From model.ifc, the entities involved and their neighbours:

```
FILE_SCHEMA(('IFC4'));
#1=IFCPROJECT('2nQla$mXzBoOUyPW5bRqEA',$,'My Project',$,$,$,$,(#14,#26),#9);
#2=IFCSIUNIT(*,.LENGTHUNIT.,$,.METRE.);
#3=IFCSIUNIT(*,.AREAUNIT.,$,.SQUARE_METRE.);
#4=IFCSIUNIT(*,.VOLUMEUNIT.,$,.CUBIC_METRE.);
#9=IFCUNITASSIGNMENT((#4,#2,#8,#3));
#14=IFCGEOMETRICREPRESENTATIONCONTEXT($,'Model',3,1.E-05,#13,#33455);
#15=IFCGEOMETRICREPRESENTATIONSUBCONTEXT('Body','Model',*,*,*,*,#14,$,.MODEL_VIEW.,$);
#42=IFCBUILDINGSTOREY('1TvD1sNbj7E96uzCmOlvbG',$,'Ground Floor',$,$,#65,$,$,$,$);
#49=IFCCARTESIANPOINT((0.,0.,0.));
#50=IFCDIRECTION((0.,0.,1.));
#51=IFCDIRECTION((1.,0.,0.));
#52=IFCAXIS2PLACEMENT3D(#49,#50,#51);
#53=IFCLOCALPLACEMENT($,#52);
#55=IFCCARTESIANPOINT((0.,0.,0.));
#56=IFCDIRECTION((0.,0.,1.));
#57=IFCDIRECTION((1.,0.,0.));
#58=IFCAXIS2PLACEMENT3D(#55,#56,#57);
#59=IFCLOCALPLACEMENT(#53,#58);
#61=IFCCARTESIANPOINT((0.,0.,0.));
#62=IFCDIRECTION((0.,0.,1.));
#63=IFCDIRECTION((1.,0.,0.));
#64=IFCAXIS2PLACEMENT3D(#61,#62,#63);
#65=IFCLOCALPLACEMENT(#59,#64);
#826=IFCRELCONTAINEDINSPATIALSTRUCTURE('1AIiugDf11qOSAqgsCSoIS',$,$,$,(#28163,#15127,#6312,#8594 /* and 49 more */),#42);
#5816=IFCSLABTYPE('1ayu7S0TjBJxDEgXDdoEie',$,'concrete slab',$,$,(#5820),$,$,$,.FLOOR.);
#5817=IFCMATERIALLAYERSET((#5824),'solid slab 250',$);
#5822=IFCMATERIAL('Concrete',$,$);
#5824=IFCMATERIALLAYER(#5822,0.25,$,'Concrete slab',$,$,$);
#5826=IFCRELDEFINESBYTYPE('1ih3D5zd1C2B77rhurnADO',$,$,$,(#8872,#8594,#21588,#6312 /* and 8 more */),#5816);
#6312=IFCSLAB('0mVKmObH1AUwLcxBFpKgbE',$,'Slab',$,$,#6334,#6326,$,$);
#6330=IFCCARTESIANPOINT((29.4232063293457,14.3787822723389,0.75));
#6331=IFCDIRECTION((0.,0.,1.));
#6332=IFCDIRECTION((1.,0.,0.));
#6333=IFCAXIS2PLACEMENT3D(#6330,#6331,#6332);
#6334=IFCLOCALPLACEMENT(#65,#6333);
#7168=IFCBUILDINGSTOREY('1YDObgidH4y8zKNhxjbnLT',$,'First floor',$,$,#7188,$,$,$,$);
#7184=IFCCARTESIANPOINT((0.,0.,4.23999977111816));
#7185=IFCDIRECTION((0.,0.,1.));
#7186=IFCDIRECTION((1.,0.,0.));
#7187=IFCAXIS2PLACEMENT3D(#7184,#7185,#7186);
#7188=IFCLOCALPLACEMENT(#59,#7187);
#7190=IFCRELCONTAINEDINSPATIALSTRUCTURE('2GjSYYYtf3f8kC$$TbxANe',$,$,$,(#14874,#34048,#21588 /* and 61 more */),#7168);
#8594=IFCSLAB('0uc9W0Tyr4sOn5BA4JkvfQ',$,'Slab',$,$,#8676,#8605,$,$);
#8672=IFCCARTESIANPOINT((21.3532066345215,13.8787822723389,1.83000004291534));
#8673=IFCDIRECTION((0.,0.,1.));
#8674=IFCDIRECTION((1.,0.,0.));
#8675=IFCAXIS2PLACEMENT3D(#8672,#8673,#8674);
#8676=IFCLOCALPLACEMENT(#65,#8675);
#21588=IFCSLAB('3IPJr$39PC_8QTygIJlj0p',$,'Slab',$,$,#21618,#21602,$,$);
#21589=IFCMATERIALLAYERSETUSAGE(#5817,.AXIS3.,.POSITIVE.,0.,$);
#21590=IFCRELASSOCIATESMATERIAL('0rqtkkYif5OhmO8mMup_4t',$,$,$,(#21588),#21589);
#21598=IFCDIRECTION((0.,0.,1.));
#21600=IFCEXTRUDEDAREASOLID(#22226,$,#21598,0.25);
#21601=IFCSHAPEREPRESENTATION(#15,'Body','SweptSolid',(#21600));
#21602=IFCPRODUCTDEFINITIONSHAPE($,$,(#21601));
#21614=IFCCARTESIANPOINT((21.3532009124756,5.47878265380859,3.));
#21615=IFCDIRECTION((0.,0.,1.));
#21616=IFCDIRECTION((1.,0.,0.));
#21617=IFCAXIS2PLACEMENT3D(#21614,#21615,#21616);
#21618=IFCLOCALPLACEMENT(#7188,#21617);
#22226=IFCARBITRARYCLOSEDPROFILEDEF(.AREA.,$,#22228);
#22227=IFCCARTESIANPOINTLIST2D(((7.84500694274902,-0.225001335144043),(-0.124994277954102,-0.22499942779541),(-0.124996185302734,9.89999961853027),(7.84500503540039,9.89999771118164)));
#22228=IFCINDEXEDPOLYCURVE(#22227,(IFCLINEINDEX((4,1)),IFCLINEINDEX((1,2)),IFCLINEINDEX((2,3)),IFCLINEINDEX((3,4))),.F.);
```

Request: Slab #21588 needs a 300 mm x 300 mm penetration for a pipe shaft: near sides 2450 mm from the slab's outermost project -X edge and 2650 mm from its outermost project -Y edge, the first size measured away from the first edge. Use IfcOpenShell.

```python
import numpy as np
import ifcopenshell
import ifcopenshell.api.feature
import ifcopenshell.api.geometry
import ifcopenshell.api.root
import ifcopenshell.geom
import ifcopenshell.util.placement
import ifcopenshell.util.representation
import ifcopenshell.util.shape
import ifcopenshell.util.unit

model = ifcopenshell.open("model.ifc")
unit_scale = ifcopenshell.util.unit.calculate_unit_scale(model)
settings = ifcopenshell.geom.settings()


def volume(element):
    """Net volume in cubic metres, openings subtracted."""
    shape = ifcopenshell.geom.create_shape(settings, element)
    return ifcopenshell.util.shape.get_volume(shape.geometry)


slab = model.by_guid("3IPJr$39PC_8QTygIJlj0p")
before = volume(slab)

# Extent in the slab's own axes, in metres. The edges named are its -X and -Y sides.
slab_shape = ifcopenshell.geom.create_shape(settings, slab)
vertices = ifcopenshell.util.shape.get_vertices(slab_shape.geometry)
x_min, y_min, bottom = vertices.min(axis=0)
top = vertices[:, 2].max()

opening = ifcopenshell.api.root.create_entity(model, ifc_class="IfcOpeningElement", name="Pipe shaft opening", predefined_type="OPENING")
context = ifcopenshell.util.representation.get_context(model, "Model", "Body", "MODEL_VIEW")
width, depth = 0.3, 0.3
outline = [(0.0, 0.0), (width, 0.0), (width, depth), (0.0, depth), (0.0, 0.0)]
# Overshoot both faces by 50 mm so the cut is clean.
shape = ifcopenshell.api.geometry.add_slab_representation(
    model, context=context, depth=top - bottom + 0.1, polyline=outline
)
ifcopenshell.api.geometry.assign_representation(model, product=opening, representation=shape)

matrix = ifcopenshell.util.placement.get_local_placement(slab.ObjectPlacement)
matrix[:, 3] = matrix @ np.append(np.array([x_min + 2.45, y_min + 2.65, bottom - 0.05]) / unit_scale, 1.0)
ifcopenshell.api.geometry.edit_object_placement(model, product=opening, matrix=matrix, is_si=False)
ifcopenshell.api.feature.add_feature(model, feature=opening, element=slab)

after = volume(slab)

print(f"slab volume {before:.3f} -> {after:.3f} m3")

model.write("model-out.ifc")
```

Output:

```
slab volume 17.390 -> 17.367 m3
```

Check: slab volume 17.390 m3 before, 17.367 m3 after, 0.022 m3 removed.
